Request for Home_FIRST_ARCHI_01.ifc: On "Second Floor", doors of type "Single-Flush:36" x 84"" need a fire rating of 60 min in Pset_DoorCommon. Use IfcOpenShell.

First a look at what the model holds.

```python
import ifcopenshell
import ifcopenshell.util.element

model = ifcopenshell.open("Home_FIRST_ARCHI_01.ifc")
print(model.schema)
storey = next(s for s in model.by_type("IfcBuildingStorey") if s.Name == "Second Floor")
doors = [e for e in ifcopenshell.util.element.get_decomposition(storey) if e.is_a("IfcDoor")]
seen = {}
for e in doors:
    element_type = ifcopenshell.util.element.get_type(e)
    key = (element_type.Name if element_type != e and element_type else None, ifcopenshell.util.element.get_pset(e, "Pset_DoorCommon", "FireRating"))
    seen[key] = seen.get(key, 0) + 1
for (name, value), count in sorted(seen.items(), key=str):
    print(count, "x", name, "|", value)
```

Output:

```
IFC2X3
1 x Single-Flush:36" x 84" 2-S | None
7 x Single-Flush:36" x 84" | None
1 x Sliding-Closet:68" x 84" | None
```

```python
import ifcopenshell
import ifcopenshell.api.pset
import ifcopenshell.util.element

model = ifcopenshell.open("Home_FIRST_ARCHI_01.ifc")

storey = next(s for s in model.by_type("IfcBuildingStorey") if s.Name == "Second Floor")
doors = [e for e in ifcopenshell.util.element.get_decomposition(storey) if e.is_a("IfcDoor")]

count = 0
for e in doors:
    element_type = ifcopenshell.util.element.get_type(e)
    if element_type in (None, e) or element_type.Name != 'Single-Flush:36" x 84"':
        continue
    # add_pset returns the element's existing set when there is one.
    pset = ifcopenshell.api.pset.add_pset(model, product=e, name="Pset_DoorCommon")
    ifcopenshell.api.pset.edit_pset(model, pset=pset, properties={"FireRating": "60 min"})
    count += 1

print(count, "doors updated")

model.write("Home_FIRST_ARCHI_01-out.ifc")
```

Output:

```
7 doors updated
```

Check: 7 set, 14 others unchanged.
